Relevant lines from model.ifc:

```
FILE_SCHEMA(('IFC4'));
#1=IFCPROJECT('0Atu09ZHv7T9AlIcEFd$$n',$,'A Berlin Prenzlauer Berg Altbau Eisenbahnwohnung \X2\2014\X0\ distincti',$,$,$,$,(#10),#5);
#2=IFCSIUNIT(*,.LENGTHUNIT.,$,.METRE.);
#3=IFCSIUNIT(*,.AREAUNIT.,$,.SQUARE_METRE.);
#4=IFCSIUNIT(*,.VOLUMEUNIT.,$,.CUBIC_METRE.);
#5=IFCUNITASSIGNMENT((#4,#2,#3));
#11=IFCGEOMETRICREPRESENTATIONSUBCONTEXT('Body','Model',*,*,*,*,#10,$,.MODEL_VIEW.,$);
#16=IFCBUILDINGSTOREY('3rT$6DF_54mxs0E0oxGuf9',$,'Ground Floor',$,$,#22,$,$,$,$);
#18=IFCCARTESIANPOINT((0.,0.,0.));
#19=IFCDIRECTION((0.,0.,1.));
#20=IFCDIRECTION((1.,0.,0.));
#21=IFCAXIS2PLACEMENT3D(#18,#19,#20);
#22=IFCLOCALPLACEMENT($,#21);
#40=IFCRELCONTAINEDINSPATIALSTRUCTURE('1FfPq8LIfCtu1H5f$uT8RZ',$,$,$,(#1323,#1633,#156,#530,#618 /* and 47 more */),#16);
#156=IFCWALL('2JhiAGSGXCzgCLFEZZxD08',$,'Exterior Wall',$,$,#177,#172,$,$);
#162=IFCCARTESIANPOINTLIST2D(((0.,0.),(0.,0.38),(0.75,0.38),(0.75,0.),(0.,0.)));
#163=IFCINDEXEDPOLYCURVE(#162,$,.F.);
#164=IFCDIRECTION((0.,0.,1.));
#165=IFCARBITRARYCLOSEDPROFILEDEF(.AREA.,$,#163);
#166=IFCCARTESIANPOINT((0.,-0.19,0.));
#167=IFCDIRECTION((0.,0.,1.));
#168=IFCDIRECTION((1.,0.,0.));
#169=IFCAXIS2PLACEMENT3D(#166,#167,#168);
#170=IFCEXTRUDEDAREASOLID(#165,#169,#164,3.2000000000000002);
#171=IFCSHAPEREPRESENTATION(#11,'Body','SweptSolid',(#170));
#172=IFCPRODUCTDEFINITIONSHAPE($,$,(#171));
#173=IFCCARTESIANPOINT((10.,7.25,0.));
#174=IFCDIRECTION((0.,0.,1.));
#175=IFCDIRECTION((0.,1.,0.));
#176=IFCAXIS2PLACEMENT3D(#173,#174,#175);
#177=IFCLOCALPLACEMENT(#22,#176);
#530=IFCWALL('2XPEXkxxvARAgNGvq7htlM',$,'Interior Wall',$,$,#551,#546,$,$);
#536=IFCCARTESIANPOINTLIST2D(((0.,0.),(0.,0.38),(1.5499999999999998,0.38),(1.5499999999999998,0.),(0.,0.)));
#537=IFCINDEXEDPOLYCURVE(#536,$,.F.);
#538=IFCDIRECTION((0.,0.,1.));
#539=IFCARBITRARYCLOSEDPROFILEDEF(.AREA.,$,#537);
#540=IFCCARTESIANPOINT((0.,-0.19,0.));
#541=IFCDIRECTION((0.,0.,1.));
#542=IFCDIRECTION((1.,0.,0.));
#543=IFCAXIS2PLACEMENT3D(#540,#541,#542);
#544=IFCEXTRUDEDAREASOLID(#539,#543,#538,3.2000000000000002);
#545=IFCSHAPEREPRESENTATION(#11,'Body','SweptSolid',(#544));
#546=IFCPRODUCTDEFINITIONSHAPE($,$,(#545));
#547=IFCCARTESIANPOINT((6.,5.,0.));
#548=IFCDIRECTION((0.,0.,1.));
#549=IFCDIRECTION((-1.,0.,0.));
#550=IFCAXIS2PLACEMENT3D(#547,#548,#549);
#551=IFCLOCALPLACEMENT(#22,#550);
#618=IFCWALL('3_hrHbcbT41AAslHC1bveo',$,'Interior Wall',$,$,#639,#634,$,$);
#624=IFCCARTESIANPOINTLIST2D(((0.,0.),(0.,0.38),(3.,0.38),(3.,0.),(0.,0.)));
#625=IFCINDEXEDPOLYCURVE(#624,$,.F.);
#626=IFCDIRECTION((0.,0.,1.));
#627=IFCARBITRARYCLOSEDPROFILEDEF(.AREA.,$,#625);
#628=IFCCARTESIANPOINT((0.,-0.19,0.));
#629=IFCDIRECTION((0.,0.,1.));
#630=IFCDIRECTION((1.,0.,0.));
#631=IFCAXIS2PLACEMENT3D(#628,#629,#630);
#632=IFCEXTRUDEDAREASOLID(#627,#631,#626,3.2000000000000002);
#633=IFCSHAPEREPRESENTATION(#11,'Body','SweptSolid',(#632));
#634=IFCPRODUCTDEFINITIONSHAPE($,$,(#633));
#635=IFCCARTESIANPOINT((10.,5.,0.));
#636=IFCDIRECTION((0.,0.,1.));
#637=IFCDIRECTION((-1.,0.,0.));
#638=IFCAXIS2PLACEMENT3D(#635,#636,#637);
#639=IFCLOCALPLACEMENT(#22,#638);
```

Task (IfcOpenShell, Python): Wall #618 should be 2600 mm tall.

```python
import ifcopenshell
import ifcopenshell.geom
import ifcopenshell.util.representation
import ifcopenshell.util.shape

model = ifcopenshell.open("model.ifc")
settings = ifcopenshell.geom.settings()


def volume(element):
    """Net volume in cubic metres, openings subtracted."""
    shape = ifcopenshell.geom.create_shape(settings, element)
    return ifcopenshell.util.shape.get_volume(shape.geometry)


wall = model.by_id(618)
before = volume(wall)

body = ifcopenshell.util.representation.get_representation(wall, "Model", "Body")
solid = body.Items[0]
old_height = solid.Depth
solid.Depth = 2.6
after = volume(wall)

print(f"height {old_height:g} -> {solid.Depth:g}, volume {before:.3f} -> {after:.3f} m3")

model.write("model_rev.ifc")
```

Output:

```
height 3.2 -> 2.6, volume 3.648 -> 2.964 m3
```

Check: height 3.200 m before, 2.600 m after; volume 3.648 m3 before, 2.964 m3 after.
